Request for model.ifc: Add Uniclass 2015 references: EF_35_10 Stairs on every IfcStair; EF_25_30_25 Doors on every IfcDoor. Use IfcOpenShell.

First a look at what the model holds.

```python
import ifcopenshell

model = ifcopenshell.open("model.ifc")
print(model.schema)
print("classifications:", [c.Name for c in model.by_type("IfcClassification")])
for ifc_class in ("IfcDoor", "IfcRoof", "IfcStair", "IfcWall", "IfcWindow"):
    print(ifc_class, len(model.by_type(ifc_class)))
```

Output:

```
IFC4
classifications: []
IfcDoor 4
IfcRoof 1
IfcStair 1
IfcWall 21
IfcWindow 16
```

```python
import ifcopenshell
import ifcopenshell.api.classification

model = ifcopenshell.open("model.ifc")

system = ifcopenshell.api.classification.add_classification(model, classification="Uniclass 2015")

codes = {
    "IfcStair": ("EF_35_10", "Stairs"),
    "IfcDoor": ("EF_25_30_25", "Doors"),
}
for ifc_class, (code, name) in codes.items():
    products = model.by_type(ifc_class)
    ifcopenshell.api.classification.add_reference(
        model, products=products, classification=system, identification=code, name=name
    )
    print(code, len(products))

model.write("model-out.ifc")
```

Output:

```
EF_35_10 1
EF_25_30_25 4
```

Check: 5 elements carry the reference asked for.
